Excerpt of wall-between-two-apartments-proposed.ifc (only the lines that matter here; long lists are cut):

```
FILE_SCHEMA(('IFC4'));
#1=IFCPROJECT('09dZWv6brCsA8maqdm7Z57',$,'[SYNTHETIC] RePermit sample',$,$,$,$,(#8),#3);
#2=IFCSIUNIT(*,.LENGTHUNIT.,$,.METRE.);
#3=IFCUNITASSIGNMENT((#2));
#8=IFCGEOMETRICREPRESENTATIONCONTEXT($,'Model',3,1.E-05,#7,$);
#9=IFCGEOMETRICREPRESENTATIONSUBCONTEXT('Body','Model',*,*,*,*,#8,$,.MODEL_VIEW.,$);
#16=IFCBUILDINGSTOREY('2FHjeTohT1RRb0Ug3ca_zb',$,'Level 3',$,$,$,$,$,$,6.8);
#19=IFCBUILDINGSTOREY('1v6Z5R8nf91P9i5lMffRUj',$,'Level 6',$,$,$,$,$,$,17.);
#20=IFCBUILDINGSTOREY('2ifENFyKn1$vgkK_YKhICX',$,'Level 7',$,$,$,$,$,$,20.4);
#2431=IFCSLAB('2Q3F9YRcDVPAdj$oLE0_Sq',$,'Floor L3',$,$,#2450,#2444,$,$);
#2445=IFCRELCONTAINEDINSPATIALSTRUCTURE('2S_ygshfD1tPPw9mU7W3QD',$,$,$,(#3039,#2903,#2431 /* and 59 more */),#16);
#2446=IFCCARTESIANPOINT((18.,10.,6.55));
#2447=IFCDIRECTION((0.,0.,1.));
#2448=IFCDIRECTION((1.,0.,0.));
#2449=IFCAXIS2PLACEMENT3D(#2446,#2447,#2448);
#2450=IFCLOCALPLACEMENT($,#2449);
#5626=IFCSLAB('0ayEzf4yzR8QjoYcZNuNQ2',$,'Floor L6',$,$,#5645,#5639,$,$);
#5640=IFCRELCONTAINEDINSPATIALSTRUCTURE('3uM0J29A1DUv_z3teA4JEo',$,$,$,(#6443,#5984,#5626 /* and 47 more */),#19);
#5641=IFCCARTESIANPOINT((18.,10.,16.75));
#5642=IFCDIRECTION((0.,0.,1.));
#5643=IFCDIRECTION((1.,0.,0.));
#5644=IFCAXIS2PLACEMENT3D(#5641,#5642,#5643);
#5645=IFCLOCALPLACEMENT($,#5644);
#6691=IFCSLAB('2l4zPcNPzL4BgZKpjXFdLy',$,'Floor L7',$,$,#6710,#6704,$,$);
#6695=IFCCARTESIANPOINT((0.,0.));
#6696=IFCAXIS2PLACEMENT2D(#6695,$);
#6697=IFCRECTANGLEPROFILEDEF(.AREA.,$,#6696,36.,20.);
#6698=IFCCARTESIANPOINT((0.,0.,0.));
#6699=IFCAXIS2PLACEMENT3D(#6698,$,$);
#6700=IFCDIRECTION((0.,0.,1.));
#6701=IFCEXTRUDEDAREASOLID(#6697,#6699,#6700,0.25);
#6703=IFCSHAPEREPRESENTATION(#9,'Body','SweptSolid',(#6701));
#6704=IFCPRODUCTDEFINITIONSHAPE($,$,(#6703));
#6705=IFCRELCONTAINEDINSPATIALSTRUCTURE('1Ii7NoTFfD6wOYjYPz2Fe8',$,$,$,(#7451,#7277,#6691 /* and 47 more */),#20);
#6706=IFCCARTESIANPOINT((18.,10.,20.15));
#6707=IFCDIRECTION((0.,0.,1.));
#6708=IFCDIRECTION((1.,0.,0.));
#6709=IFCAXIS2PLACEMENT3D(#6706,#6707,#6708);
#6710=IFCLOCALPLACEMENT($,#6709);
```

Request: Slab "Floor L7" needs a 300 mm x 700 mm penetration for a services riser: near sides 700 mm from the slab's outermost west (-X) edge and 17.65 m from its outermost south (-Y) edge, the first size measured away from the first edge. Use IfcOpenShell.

```python
import numpy as np
import ifcopenshell
import ifcopenshell.api.feature
import ifcopenshell.api.geometry
import ifcopenshell.api.root
import ifcopenshell.geom
import ifcopenshell.util.placement
import ifcopenshell.util.representation
import ifcopenshell.util.shape
import ifcopenshell.util.unit

model = ifcopenshell.open("wall-between-two-apartments-proposed.ifc")
unit_scale = ifcopenshell.util.unit.calculate_unit_scale(model)
settings = ifcopenshell.geom.settings()


def volume(element):
    """Net volume in cubic metres, openings subtracted."""
    shape = ifcopenshell.geom.create_shape(settings, element)
    return ifcopenshell.util.shape.get_volume(shape.geometry)


slab = model.by_guid("2l4zPcNPzL4BgZKpjXFdLy")
before = volume(slab)

# Extent in the slab's own axes, in metres. The edges named are its -X and -Y sides.
slab_shape = ifcopenshell.geom.create_shape(settings, slab)
vertices = ifcopenshell.util.shape.get_vertices(slab_shape.geometry)
x_min, y_min, bottom = vertices.min(axis=0)
top = vertices[:, 2].max()

opening = ifcopenshell.api.root.create_entity(model, ifc_class="IfcOpeningElement", name="Services riser opening", predefined_type="OPENING")
context = ifcopenshell.util.representation.get_context(model, "Model", "Body", "MODEL_VIEW")
width, depth = 0.3, 0.7
outline = [(0.0, 0.0), (width, 0.0), (width, depth), (0.0, depth), (0.0, 0.0)]
# Overshoot both faces by 50 mm so the cut is clean.
shape = ifcopenshell.api.geometry.add_slab_representation(
    model, context=context, depth=top - bottom + 0.1, polyline=outline
)
ifcopenshell.api.geometry.assign_representation(model, product=opening, representation=shape)

matrix = ifcopenshell.util.placement.get_local_placement(slab.ObjectPlacement)
matrix[:, 3] = matrix @ np.append(np.array([x_min + 0.7, y_min + 17.65, bottom - 0.05]) / unit_scale, 1.0)
ifcopenshell.api.geometry.edit_object_placement(model, product=opening, matrix=matrix, is_si=False)
ifcopenshell.api.feature.add_feature(model, feature=opening, element=slab)

after = volume(slab)

print(f"slab volume {before:.3f} -> {after:.3f} m3")

model.write("wall-between-two-apartments-proposed_edited.ifc")
```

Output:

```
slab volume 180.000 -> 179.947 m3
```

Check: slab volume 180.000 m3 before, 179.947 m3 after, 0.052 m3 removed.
